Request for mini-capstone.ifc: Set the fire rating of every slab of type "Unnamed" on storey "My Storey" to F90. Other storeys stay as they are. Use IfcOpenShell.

First a look at what the model holds.

```python
import ifcopenshell
import ifcopenshell.util.element

model = ifcopenshell.open("mini-capstone.ifc")
print(model.schema)
storey = next(s for s in model.by_type("IfcBuildingStorey") if s.Name == "My Storey")
slabs = [e for e in ifcopenshell.util.element.get_decomposition(storey) if e.is_a("IfcSlab")]
seen = {}
for e in slabs:
    element_type = ifcopenshell.util.element.get_type(e)
    key = (element_type.Name if element_type != e and element_type else None, ifcopenshell.util.element.get_pset(e, "Pset_SlabCommon", "FireRating"))
    seen[key] = seen.get(key, 0) + 1
for (name, value), count in sorted(seen.items(), key=str):
    print(count, "x", name, "|", value)
```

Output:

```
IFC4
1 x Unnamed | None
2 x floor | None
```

```python
import ifcopenshell
import ifcopenshell.api.pset
import ifcopenshell.util.element

model = ifcopenshell.open("mini-capstone.ifc")

storey = next(s for s in model.by_type("IfcBuildingStorey") if s.Name == "My Storey")
slabs = [e for e in ifcopenshell.util.element.get_decomposition(storey) if e.is_a("IfcSlab")]

count = 0
for e in slabs:
    element_type = ifcopenshell.util.element.get_type(e)
    if element_type in (None, e) or element_type.Name != "Unnamed":
        continue
    # add_pset returns the element's existing set when there is one.
    pset = ifcopenshell.api.pset.add_pset(model, product=e, name="Pset_SlabCommon")
    ifcopenshell.api.pset.edit_pset(model, pset=pset, properties={"FireRating": "F90"})
    count += 1

print(count, "slabs updated")

model.write("mini-capstone_v2.ifc")
```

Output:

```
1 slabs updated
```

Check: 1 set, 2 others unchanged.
